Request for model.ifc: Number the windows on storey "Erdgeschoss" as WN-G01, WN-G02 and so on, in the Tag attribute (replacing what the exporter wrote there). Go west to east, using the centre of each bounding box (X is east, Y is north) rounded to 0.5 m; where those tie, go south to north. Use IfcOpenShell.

First a look at what the model holds.

```python
import ifcopenshell
import ifcopenshell.util.element
import ifcopenshell.util.placement

model = ifcopenshell.open("model.ifc")
print(model.schema)
storey = next(s for s in model.by_type("IfcBuildingStorey") if s.Name == "Erdgeschoss")
windows = [e for e in ifcopenshell.util.element.get_decomposition(storey) if e.is_a("IfcWindow")]
for e in sorted(windows, key=lambda e: e.id()):
    origin = ifcopenshell.util.placement.get_local_placement(e.ObjectPlacement)[:3, 3]
    print(e.id(), e.Tag, e.Name, origin.round(2) + 0.0, sep=" | ")
```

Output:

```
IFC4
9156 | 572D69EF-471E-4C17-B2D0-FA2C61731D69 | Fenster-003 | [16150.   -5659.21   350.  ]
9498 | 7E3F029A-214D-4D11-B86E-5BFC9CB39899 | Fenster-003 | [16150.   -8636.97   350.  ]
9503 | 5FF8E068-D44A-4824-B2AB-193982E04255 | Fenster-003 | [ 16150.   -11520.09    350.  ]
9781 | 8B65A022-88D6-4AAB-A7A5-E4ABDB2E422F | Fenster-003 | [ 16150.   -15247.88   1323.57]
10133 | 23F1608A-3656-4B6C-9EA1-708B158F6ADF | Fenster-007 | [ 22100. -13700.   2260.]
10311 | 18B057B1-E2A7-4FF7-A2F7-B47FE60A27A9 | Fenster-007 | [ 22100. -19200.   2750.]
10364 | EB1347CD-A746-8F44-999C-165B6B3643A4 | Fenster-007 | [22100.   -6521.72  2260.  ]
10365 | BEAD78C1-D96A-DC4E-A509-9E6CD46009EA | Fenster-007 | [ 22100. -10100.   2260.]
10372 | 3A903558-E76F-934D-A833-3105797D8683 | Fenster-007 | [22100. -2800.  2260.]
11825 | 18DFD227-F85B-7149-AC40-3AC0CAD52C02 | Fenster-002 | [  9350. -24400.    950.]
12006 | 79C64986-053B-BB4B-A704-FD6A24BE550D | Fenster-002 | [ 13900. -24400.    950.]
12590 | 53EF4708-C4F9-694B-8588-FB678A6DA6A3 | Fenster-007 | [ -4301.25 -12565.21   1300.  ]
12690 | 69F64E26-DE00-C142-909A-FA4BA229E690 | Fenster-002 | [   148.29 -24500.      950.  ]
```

```python
import ifcopenshell
import ifcopenshell.geom
import ifcopenshell.util.element
import ifcopenshell.util.shape

model = ifcopenshell.open("model.ifc")
settings = ifcopenshell.geom.settings()
settings.set("use-world-coords", True)


def centre(element):
    shape = ifcopenshell.geom.create_shape(settings, element)
    return ifcopenshell.util.shape.get_bbox_centroid(shape.geometry)


storey = next(s for s in model.by_type("IfcBuildingStorey") if s.Name == "Erdgeschoss")
windows = [e for e in ifcopenshell.util.element.get_decomposition(storey) if e.is_a("IfcWindow")]

# Insertion points can sit at a corner or the storey origin, so sort by the geometry (in metres).
centres = {e: centre(e) for e in windows}
windows.sort(key=lambda e: (round(centres[e][0] / 0.5), centres[e][1]))

for i, e in enumerate(windows, start=1):
    number = f"WN-G{i:02d}"
    e.Tag = number
    print(e.id(), number)

model.write("model_v2.ifc")
```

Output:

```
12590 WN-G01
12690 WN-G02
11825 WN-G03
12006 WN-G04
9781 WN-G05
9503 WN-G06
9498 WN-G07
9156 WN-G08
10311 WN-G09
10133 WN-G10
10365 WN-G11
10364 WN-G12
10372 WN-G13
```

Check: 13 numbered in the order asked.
